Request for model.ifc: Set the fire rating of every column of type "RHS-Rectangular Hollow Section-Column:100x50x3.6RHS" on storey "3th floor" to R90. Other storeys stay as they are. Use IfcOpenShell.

First a look at what the model holds.

```python
import ifcopenshell
import ifcopenshell.util.element

model = ifcopenshell.open("model.ifc")
print(model.schema)
storey = next(s for s in model.by_type("IfcBuildingStorey") if s.Name == "3th floor")
columns = [e for e in ifcopenshell.util.element.get_decomposition(storey) if e.is_a("IfcColumn")]
seen = {}
for e in columns:
    element_type = ifcopenshell.util.element.get_type(e)
    key = (element_type.Name if element_type != e and element_type else None, ifcopenshell.util.element.get_pset(e, "Pset_ColumnCommon", "FireRating"))
    seen[key] = seen.get(key, 0) + 1
for (name, value), count in sorted(seen.items(), key=str):
    print(count, "x", name, "|", value)
```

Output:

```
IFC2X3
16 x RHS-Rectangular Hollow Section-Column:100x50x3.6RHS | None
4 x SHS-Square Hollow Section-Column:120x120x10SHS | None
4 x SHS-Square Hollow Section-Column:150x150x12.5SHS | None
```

```python
import ifcopenshell
import ifcopenshell.api.pset
import ifcopenshell.util.element

model = ifcopenshell.open("model.ifc")

storey = next(s for s in model.by_type("IfcBuildingStorey") if s.Name == "3th floor")
columns = [e for e in ifcopenshell.util.element.get_decomposition(storey) if e.is_a("IfcColumn")]

count = 0
for e in columns:
    element_type = ifcopenshell.util.element.get_type(e)
    if element_type in (None, e) or element_type.Name != "RHS-Rectangular Hollow Section-Column:100x50x3.6RHS":
        continue
    # add_pset returns the element's existing set when there is one.
    pset = ifcopenshell.api.pset.add_pset(model, product=e, name="Pset_ColumnCommon")
    ifcopenshell.api.pset.edit_pset(model, pset=pset, properties={"FireRating": "R90"})
    count += 1

print(count, "columns updated")

model.write("model_v2.ifc")
```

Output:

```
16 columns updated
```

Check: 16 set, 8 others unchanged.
